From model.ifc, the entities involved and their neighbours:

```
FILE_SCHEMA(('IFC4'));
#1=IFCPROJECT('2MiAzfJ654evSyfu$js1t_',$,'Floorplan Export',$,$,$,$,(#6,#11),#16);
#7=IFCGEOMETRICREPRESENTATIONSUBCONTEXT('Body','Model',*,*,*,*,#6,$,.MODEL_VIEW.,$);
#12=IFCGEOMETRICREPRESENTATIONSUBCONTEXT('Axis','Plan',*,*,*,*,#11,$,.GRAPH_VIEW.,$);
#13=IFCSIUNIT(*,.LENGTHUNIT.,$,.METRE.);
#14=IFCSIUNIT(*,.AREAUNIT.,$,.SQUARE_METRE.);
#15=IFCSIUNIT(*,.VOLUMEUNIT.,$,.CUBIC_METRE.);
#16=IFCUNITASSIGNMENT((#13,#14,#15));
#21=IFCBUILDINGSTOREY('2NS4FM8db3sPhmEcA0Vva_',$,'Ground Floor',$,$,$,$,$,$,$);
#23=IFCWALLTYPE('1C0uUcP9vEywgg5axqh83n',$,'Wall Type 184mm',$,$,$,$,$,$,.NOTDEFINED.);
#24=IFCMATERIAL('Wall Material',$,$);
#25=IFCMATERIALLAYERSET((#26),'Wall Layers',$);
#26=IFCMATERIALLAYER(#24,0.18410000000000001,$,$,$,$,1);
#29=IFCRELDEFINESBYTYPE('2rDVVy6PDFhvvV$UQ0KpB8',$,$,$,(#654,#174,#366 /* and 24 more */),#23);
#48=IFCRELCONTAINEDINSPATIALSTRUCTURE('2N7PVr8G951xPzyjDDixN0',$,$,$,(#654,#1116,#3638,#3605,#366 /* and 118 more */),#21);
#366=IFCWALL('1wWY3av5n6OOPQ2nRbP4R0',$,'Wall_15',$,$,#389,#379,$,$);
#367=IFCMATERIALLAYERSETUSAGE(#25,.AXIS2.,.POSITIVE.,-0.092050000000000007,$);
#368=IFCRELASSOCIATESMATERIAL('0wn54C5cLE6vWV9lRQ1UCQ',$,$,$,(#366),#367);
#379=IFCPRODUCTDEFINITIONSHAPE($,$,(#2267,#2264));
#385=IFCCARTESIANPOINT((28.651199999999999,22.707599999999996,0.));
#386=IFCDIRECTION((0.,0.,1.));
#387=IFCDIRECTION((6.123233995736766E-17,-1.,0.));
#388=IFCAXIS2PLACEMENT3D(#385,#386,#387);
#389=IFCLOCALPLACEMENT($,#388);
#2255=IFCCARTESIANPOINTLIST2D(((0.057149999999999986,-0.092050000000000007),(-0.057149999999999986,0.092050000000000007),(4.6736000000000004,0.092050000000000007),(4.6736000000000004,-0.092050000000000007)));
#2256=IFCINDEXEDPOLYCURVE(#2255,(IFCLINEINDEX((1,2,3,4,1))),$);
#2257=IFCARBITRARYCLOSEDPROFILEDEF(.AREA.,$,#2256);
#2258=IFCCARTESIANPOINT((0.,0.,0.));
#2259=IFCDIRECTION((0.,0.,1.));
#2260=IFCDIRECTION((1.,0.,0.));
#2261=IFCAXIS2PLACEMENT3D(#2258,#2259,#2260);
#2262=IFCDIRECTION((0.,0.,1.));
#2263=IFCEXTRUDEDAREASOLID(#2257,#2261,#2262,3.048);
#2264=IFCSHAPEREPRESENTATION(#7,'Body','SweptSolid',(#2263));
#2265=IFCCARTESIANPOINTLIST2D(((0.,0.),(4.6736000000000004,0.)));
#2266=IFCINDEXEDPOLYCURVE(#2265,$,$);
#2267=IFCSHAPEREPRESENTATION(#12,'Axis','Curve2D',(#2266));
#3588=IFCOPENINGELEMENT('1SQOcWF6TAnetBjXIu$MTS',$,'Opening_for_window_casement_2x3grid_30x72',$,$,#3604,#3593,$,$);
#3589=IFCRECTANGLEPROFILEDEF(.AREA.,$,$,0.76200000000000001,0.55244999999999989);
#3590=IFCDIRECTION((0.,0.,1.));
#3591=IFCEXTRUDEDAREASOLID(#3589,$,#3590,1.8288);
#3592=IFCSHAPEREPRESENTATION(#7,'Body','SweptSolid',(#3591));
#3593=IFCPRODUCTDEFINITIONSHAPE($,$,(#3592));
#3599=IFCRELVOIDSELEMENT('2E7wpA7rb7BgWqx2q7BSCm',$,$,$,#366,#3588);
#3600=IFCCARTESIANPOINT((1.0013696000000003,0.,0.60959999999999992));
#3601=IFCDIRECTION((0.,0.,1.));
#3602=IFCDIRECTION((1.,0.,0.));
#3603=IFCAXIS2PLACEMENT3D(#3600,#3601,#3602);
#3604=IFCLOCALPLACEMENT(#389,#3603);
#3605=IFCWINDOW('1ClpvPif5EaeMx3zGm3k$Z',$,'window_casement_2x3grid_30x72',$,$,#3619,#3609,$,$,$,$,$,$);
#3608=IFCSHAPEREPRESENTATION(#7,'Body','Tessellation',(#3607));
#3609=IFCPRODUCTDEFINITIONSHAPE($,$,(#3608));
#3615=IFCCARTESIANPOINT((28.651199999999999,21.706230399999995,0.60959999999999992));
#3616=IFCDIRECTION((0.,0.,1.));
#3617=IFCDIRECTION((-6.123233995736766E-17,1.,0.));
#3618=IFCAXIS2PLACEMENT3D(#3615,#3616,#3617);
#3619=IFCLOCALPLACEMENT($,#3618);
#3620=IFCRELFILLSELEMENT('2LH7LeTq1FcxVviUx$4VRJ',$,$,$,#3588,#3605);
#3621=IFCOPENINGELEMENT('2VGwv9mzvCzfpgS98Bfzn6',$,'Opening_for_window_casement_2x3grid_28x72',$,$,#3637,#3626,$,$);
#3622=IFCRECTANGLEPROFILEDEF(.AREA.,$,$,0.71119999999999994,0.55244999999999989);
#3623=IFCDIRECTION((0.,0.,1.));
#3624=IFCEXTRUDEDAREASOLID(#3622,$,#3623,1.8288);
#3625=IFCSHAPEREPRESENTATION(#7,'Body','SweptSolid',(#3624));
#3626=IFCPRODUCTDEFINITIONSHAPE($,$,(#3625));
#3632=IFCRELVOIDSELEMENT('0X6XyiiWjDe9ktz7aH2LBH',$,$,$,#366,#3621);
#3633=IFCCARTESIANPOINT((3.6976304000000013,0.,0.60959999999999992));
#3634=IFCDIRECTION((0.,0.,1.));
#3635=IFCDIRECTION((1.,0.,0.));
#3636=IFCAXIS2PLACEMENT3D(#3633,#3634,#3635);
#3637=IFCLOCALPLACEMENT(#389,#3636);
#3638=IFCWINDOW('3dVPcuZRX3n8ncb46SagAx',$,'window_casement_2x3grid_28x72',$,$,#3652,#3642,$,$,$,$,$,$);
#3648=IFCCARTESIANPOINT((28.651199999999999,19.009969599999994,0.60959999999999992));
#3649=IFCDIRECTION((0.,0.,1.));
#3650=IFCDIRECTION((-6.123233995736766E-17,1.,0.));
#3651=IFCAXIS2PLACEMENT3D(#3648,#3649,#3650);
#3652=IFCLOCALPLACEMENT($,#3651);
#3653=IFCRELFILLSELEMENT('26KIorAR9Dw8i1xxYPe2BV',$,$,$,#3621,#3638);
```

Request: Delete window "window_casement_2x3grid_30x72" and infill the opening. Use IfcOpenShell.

```python
import ifcopenshell
import ifcopenshell.api.feature
import ifcopenshell.api.root
import ifcopenshell.geom
import ifcopenshell.util.shape

model = ifcopenshell.open("model.ifc")
settings = ifcopenshell.geom.settings()


def volume(element):
    """Net volume in cubic metres, openings subtracted."""
    shape = ifcopenshell.geom.create_shape(settings, element)
    return ifcopenshell.util.shape.get_volume(shape.geometry)


window = model.by_id(3605)
opening = window.FillsVoids[0].RelatingOpeningElement
wall = opening.VoidsElements[0].RelatingBuildingElement
before = volume(wall)

ifcopenshell.api.root.remove_product(model, product=window)
ifcopenshell.api.feature.remove_feature(model, feature=opening)

after = volume(wall)

print(f"wall volume {before:.3f} -> {after:.3f} m3")

model.write("model-out.ifc")
```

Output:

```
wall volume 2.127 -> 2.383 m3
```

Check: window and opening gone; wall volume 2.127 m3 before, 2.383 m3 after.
